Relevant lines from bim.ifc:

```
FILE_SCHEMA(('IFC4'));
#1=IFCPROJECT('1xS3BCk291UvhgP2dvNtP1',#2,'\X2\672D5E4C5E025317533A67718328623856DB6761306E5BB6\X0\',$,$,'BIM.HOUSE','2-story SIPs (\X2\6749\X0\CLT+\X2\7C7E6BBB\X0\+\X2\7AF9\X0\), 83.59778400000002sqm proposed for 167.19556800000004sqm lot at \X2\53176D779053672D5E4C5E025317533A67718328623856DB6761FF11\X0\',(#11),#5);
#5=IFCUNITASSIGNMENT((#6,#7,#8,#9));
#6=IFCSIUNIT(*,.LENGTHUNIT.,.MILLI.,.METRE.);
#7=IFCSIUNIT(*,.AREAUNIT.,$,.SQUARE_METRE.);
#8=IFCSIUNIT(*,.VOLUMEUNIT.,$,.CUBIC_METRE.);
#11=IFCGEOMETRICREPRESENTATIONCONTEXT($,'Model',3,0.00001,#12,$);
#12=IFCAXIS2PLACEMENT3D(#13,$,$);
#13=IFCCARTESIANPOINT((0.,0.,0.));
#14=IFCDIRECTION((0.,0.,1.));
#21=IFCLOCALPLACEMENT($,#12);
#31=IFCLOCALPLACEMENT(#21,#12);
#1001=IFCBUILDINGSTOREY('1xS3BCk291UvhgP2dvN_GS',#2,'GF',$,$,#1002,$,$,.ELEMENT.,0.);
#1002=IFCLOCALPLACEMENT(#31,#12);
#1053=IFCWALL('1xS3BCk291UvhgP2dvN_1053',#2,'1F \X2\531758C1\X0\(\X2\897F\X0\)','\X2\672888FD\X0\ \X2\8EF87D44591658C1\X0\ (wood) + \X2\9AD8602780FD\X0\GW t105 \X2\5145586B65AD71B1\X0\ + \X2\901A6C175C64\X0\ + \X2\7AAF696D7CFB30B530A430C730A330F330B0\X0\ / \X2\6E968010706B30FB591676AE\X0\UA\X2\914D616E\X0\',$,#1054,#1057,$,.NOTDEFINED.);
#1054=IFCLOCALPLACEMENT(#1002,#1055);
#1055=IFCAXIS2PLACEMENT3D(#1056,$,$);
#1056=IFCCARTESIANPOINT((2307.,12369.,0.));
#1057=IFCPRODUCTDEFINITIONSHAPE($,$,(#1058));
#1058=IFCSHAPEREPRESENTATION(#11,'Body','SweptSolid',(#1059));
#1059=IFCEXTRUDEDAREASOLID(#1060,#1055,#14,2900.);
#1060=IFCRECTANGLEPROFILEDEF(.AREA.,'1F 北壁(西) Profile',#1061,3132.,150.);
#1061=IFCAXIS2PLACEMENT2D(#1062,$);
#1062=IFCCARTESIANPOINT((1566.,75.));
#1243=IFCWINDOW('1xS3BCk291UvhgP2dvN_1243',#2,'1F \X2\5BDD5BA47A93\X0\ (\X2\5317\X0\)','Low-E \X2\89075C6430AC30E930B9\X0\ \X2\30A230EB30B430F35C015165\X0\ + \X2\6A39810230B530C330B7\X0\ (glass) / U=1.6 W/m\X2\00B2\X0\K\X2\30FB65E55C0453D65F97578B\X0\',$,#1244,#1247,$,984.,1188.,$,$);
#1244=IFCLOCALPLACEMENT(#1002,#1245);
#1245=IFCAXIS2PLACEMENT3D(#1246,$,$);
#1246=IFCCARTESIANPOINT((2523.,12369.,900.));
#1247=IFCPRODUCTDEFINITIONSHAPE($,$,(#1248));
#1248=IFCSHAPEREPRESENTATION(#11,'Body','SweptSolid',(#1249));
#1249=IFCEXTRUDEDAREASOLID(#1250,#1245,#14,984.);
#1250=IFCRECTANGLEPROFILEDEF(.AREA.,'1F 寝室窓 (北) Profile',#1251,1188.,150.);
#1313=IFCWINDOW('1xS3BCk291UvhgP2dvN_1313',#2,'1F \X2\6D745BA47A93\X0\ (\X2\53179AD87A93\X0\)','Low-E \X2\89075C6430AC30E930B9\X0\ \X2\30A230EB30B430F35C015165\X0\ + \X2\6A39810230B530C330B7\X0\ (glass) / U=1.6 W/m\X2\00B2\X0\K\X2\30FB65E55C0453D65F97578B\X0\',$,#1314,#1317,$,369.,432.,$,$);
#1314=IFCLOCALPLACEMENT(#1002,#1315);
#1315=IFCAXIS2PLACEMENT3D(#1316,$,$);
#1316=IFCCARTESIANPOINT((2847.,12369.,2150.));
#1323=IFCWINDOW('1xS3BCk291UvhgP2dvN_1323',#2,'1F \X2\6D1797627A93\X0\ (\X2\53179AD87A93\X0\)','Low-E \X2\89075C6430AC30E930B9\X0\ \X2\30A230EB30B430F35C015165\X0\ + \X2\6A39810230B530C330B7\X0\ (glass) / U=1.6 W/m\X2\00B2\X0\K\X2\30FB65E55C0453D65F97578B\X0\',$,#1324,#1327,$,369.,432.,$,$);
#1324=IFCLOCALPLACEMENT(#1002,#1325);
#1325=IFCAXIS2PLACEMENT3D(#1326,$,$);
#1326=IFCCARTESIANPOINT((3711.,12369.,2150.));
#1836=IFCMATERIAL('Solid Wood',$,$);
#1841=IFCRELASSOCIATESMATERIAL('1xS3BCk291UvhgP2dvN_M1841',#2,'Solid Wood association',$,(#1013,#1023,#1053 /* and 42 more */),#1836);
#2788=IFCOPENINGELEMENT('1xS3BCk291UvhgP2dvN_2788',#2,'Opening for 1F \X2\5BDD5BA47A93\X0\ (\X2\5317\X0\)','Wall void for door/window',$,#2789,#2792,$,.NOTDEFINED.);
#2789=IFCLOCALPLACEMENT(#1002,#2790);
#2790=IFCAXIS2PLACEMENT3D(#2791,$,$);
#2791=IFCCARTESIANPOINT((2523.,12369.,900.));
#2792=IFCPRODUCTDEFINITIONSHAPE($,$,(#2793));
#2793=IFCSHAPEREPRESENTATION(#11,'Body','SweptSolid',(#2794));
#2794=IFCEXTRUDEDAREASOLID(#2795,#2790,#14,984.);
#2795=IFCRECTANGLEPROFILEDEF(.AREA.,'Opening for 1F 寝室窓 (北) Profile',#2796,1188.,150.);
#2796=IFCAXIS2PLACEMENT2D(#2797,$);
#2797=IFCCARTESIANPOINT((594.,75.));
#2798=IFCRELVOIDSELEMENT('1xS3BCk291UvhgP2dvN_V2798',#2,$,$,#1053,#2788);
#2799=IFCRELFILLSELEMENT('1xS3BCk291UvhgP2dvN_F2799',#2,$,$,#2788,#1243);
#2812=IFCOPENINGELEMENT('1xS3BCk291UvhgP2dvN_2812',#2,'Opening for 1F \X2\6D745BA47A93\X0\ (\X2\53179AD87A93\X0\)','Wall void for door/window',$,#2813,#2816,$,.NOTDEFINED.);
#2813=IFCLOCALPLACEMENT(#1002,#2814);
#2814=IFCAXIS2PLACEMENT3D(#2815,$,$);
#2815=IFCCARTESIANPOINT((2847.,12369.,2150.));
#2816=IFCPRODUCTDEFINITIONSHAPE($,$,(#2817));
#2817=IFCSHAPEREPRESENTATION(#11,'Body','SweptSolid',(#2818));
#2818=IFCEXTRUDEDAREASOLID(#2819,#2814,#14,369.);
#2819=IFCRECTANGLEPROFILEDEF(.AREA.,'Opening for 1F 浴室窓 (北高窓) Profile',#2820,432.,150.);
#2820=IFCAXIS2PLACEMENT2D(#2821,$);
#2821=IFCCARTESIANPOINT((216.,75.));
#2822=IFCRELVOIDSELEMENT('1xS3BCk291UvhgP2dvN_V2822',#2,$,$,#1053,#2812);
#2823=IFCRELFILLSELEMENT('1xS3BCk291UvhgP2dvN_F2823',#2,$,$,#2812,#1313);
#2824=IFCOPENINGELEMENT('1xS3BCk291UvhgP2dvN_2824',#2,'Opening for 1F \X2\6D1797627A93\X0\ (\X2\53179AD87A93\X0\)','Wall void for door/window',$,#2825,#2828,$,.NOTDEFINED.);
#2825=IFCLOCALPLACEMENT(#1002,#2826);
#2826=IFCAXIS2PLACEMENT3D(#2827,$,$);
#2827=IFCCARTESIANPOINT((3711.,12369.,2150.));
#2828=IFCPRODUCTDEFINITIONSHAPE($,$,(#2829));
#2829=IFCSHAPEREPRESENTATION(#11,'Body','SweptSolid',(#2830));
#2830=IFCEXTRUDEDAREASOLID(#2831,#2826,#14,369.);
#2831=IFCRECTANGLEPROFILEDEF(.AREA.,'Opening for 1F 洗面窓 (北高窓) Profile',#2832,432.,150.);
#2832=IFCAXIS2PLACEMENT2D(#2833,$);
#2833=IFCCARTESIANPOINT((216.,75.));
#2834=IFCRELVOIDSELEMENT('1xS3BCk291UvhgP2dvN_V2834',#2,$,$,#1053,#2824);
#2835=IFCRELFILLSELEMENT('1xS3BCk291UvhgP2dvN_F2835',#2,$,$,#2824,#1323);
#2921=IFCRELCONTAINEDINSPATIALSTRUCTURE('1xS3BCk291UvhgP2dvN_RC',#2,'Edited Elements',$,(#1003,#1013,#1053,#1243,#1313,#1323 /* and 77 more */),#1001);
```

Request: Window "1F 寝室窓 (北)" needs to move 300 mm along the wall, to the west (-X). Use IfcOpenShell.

```python
import ifcopenshell
import ifcopenshell.api.geometry
import ifcopenshell.util.placement
import ifcopenshell.util.unit

model = ifcopenshell.open("bim.ifc")
unit_scale = ifcopenshell.util.unit.calculate_unit_scale(model)

window = model.by_guid("1xS3BCk291UvhgP2dvN_1243")
opening = window.FillsVoids[0].RelatingOpeningElement
wall = opening.VoidsElements[0].RelatingBuildingElement

wall_matrix = ifcopenshell.util.placement.get_local_placement(wall.ObjectPlacement)
shift = wall_matrix[:3, 0] * -0.3 / unit_scale
before = ifcopenshell.util.placement.get_local_placement(window.ObjectPlacement)[:3, 3].copy()

# The window is not placed relative to its opening, so move both.
for product in (opening, window):
    matrix = ifcopenshell.util.placement.get_local_placement(product.ObjectPlacement)
    matrix[:3, 3] += shift
    ifcopenshell.api.geometry.edit_object_placement(model, product=product, matrix=matrix, is_si=False)

after = ifcopenshell.util.placement.get_local_placement(window.ObjectPlacement)[:3, 3]
print("window moved by", (after - before).round(3) + 0.0)

model.write("bim-out.ifc")
```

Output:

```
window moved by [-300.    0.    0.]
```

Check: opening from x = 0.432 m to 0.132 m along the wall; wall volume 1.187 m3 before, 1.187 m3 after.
